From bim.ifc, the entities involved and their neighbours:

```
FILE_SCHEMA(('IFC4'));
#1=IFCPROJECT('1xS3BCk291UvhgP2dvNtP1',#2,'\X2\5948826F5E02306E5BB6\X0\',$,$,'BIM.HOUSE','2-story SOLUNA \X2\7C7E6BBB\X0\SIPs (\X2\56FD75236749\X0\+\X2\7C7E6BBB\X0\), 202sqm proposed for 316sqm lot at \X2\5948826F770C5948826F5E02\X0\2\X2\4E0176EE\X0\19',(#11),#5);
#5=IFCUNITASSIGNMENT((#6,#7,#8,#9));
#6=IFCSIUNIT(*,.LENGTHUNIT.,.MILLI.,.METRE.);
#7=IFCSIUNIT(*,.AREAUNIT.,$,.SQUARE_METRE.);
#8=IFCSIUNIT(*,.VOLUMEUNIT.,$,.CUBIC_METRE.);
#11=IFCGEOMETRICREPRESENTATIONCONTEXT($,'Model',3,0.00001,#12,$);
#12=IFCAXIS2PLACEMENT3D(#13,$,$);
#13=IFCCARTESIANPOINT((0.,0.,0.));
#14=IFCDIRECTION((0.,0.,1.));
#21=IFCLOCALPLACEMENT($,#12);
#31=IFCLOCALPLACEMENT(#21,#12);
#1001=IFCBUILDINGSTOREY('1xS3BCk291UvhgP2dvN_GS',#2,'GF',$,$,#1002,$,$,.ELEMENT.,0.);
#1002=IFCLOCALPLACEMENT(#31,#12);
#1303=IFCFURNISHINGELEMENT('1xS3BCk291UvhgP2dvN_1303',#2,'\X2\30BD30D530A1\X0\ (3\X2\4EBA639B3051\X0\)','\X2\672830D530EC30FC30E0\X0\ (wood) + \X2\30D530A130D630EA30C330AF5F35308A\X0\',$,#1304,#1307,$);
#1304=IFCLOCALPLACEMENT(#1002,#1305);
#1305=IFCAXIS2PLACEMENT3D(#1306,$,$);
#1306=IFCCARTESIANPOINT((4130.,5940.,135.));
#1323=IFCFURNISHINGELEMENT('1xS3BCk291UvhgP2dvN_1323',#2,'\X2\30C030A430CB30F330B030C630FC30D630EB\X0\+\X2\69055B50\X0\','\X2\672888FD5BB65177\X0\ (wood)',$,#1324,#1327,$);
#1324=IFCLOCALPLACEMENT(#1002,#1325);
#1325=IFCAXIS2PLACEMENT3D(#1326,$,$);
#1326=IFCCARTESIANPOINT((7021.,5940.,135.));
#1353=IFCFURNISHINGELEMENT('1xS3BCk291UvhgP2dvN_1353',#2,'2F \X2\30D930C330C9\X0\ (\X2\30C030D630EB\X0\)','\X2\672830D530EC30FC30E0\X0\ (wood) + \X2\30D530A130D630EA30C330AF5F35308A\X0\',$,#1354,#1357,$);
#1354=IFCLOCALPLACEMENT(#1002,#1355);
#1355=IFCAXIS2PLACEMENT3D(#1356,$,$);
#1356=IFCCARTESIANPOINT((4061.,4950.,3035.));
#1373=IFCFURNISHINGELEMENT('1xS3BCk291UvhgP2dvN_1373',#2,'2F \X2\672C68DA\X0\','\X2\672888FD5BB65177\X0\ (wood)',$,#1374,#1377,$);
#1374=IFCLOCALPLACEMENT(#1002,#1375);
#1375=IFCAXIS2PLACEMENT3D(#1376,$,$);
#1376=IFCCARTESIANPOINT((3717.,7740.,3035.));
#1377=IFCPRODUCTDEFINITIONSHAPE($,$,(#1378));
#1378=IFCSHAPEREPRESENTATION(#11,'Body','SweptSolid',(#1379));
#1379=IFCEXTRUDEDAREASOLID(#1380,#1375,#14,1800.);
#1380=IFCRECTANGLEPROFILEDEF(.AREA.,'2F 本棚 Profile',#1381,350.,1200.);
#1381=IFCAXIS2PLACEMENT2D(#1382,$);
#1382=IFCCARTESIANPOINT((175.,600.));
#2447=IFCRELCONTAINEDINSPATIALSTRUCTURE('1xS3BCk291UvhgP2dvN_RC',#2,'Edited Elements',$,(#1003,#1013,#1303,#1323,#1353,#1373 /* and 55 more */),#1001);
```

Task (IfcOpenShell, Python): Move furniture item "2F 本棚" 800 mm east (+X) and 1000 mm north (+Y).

```python
import ifcopenshell
import ifcopenshell.api.geometry
import ifcopenshell.util.placement
import ifcopenshell.util.unit

model = ifcopenshell.open("bim.ifc")
unit_scale = ifcopenshell.util.unit.calculate_unit_scale(model)

item = model.by_guid("1xS3BCk291UvhgP2dvN_1373")
matrix = ifcopenshell.util.placement.get_local_placement(item.ObjectPlacement)
matrix[0, 3] += 0.8 / unit_scale
matrix[1, 3] += 1 / unit_scale
ifcopenshell.api.geometry.edit_object_placement(model, product=item, matrix=matrix, is_si=False)

print(ifcopenshell.util.placement.get_local_placement(item.ObjectPlacement).round(3) + 0.0)

model.write("bim_edited.ifc")
```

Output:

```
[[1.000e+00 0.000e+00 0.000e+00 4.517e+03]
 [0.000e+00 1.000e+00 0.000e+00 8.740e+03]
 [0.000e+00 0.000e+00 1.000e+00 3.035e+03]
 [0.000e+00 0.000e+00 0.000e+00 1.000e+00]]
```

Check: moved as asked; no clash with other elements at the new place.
